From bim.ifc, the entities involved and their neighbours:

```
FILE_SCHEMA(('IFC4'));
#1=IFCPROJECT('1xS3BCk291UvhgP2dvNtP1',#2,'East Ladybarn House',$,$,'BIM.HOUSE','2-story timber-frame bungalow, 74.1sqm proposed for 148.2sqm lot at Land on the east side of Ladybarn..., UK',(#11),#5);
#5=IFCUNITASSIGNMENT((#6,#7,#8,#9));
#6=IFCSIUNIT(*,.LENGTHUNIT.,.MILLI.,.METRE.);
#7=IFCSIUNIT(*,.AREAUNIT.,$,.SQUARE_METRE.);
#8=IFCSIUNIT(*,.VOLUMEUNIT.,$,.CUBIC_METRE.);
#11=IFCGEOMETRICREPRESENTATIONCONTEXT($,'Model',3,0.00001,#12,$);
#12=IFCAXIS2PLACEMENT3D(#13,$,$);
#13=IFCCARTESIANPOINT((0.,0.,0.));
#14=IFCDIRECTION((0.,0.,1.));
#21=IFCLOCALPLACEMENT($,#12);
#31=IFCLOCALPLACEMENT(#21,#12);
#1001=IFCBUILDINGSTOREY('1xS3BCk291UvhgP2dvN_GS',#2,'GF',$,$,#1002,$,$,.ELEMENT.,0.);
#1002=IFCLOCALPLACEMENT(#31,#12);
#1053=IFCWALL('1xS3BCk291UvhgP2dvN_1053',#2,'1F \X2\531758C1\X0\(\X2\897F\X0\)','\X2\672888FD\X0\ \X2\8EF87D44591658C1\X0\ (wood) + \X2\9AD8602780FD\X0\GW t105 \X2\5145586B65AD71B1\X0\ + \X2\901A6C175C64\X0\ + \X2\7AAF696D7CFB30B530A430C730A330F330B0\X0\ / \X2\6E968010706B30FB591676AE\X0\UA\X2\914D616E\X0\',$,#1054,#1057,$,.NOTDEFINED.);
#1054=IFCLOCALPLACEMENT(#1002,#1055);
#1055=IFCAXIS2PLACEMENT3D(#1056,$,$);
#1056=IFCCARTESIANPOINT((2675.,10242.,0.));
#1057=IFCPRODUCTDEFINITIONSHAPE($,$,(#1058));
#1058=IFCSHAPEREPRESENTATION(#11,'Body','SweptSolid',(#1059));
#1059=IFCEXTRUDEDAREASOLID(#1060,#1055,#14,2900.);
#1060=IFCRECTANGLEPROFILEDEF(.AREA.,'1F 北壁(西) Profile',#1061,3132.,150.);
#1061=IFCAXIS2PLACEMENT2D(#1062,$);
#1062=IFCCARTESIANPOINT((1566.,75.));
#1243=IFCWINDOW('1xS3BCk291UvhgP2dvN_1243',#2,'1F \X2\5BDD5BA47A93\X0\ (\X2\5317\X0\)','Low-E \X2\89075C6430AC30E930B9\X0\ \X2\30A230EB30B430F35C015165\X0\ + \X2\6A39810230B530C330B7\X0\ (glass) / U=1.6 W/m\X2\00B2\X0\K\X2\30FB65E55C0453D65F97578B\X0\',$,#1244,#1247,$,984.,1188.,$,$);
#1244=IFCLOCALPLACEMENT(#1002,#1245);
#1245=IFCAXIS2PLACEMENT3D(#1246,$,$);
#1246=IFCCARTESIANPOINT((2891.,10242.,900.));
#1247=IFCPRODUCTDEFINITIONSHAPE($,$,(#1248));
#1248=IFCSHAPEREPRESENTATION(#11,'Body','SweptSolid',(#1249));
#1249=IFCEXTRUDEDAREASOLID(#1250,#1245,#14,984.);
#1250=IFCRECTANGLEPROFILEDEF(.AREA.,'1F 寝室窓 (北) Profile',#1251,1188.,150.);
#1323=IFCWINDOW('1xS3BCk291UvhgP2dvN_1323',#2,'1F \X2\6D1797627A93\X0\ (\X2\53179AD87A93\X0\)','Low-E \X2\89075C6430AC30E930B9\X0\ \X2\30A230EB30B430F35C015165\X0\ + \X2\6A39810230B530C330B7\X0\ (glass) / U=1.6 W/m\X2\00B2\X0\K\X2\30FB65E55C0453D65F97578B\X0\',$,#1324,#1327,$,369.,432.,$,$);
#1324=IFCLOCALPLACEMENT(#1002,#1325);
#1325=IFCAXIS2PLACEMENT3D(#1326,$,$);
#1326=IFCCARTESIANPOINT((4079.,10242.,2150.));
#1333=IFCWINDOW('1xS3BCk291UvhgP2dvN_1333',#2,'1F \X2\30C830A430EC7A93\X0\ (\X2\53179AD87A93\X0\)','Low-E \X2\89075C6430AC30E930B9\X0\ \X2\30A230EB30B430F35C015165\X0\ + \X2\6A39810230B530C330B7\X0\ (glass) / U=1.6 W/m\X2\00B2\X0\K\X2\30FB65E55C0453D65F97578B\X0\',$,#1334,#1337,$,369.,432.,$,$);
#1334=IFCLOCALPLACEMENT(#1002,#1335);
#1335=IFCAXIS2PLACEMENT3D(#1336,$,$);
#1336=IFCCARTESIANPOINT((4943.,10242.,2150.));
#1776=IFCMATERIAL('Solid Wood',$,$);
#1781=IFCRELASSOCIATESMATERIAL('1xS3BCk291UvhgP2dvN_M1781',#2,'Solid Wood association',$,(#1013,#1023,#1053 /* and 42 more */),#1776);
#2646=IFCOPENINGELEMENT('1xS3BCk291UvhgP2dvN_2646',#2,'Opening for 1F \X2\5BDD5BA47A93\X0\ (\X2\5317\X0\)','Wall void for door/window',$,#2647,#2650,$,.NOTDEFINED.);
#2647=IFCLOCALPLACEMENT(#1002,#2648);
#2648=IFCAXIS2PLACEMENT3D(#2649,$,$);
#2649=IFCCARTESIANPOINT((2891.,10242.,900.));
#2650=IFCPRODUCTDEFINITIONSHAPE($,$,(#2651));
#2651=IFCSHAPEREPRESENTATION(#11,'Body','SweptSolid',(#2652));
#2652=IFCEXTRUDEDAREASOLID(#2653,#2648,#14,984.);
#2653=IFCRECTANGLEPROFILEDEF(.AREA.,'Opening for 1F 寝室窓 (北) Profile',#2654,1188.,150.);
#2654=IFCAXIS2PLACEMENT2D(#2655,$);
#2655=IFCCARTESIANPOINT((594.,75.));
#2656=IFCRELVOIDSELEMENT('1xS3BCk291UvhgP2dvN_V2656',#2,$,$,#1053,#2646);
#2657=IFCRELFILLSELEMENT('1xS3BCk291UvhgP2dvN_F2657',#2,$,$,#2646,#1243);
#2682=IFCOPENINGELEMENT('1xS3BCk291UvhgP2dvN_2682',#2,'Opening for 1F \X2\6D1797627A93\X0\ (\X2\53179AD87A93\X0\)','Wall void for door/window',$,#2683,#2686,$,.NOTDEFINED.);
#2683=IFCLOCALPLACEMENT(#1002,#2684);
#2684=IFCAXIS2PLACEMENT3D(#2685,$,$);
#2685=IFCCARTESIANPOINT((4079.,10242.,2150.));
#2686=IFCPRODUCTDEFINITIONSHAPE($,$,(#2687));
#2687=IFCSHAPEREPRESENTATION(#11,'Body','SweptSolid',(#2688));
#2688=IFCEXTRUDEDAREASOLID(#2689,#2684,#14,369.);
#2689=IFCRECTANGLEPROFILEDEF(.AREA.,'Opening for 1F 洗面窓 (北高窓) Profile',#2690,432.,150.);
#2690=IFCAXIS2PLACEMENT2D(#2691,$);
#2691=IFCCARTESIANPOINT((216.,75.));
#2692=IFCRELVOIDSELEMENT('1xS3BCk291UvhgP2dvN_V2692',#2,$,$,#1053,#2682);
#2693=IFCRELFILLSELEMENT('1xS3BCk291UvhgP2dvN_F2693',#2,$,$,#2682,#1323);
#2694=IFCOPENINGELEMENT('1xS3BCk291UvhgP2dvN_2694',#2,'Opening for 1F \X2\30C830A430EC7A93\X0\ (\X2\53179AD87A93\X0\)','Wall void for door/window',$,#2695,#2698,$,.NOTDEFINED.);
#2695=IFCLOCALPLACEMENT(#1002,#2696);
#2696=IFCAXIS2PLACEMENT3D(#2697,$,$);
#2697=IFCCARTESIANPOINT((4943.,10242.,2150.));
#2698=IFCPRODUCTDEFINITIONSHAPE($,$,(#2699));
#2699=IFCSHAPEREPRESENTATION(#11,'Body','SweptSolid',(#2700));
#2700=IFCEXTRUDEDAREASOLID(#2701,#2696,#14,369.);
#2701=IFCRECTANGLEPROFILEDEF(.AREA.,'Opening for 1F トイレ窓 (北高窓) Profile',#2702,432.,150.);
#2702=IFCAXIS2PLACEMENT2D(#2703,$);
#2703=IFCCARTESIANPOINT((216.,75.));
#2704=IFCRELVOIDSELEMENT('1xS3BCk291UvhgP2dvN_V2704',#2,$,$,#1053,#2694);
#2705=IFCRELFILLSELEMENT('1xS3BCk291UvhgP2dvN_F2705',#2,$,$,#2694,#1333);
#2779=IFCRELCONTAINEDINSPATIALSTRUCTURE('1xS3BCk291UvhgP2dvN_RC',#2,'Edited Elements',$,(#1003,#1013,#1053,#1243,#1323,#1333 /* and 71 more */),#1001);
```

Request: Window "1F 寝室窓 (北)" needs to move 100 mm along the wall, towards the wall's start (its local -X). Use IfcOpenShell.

```python
import ifcopenshell
import ifcopenshell.api.geometry
import ifcopenshell.util.placement
import ifcopenshell.util.unit

model = ifcopenshell.open("bim.ifc")
unit_scale = ifcopenshell.util.unit.calculate_unit_scale(model)

window = model.by_guid("1xS3BCk291UvhgP2dvN_1243")
opening = window.FillsVoids[0].RelatingOpeningElement
wall = opening.VoidsElements[0].RelatingBuildingElement

wall_matrix = ifcopenshell.util.placement.get_local_placement(wall.ObjectPlacement)
shift = wall_matrix[:3, 0] * -0.1 / unit_scale
before = ifcopenshell.util.placement.get_local_placement(window.ObjectPlacement)[:3, 3].copy()

# The window is not placed relative to its opening, so move both.
for product in (opening, window):
    matrix = ifcopenshell.util.placement.get_local_placement(product.ObjectPlacement)
    matrix[:3, 3] += shift
    ifcopenshell.api.geometry.edit_object_placement(model, product=product, matrix=matrix, is_si=False)

after = ifcopenshell.util.placement.get_local_placement(window.ObjectPlacement)[:3, 3]
print("window moved by", (after - before).round(3) + 0.0)

model.write("bim_edited.ifc")
```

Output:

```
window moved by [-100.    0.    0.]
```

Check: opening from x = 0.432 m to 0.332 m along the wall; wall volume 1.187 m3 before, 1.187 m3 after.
